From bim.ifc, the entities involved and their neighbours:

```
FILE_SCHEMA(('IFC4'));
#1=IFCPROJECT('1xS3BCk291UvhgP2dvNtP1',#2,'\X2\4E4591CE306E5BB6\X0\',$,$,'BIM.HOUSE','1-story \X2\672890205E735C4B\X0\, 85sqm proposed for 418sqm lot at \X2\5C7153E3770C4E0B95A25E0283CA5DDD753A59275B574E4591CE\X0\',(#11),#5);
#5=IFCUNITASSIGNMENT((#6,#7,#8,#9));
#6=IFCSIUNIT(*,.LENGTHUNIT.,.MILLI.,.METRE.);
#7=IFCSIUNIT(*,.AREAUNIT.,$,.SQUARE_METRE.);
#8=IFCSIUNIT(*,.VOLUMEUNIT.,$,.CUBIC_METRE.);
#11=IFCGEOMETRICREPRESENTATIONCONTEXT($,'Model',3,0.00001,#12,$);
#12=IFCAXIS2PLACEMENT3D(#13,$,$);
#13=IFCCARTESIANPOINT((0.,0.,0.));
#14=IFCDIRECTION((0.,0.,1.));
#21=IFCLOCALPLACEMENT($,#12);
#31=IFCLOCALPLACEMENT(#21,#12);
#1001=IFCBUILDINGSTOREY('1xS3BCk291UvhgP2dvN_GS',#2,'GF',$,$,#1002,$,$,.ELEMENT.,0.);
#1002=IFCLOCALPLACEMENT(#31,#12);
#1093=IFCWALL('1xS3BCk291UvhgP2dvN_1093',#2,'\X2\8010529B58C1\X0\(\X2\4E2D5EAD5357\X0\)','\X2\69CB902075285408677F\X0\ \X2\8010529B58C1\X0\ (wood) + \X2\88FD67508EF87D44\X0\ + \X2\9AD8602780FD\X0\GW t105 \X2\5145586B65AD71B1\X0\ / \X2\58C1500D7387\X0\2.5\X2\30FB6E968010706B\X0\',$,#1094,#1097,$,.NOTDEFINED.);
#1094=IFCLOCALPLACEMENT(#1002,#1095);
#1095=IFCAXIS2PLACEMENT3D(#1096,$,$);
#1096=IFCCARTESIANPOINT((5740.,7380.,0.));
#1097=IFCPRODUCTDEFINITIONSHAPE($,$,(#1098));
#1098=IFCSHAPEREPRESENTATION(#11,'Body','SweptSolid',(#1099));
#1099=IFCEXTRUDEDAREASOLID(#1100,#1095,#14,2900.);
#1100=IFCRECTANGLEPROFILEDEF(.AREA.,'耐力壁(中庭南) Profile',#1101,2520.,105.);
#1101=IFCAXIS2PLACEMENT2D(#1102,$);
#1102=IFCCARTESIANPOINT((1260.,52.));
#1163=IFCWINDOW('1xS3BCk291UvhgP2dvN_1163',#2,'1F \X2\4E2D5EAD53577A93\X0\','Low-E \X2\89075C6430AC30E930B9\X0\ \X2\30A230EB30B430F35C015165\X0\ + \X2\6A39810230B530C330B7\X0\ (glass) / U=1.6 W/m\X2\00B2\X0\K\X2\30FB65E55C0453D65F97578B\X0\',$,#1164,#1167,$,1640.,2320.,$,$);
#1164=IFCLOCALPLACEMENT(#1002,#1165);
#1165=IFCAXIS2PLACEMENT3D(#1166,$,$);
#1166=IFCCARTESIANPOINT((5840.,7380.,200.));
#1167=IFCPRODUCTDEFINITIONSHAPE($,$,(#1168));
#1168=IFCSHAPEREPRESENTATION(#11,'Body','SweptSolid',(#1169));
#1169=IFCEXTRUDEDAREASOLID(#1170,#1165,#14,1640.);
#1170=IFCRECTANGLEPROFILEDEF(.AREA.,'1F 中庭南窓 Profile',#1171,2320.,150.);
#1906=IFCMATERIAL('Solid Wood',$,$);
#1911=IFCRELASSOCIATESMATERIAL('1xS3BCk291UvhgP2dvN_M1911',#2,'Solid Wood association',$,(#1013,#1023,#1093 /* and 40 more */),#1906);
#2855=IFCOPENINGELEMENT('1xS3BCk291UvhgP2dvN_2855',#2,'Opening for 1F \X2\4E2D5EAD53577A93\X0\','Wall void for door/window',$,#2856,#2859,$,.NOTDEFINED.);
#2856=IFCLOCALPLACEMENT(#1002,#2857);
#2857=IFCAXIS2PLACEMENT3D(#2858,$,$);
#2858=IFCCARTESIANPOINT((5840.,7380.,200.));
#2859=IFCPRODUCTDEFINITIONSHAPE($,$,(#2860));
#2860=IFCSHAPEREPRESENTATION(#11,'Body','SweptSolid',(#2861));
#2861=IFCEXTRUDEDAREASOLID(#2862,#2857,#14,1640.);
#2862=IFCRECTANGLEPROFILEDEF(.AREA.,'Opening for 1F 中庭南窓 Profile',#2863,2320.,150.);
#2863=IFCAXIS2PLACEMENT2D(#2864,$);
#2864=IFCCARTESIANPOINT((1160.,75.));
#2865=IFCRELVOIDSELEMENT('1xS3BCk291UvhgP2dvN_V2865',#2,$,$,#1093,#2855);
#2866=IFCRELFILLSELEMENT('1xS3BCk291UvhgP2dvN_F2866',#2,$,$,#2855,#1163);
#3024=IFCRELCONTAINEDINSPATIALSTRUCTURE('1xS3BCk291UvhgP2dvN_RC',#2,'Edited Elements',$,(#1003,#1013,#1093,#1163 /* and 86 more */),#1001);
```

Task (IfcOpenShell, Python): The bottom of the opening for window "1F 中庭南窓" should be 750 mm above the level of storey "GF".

```python
import numpy as np
import ifcopenshell
import ifcopenshell.api.geometry
import ifcopenshell.geom
import ifcopenshell.util.element
import ifcopenshell.util.placement
import ifcopenshell.util.shape
import ifcopenshell.util.unit

model = ifcopenshell.open("bim.ifc")
unit_scale = ifcopenshell.util.unit.calculate_unit_scale(model)

window = model.by_id(1163)
opening = window.FillsVoids[0].RelatingOpeningElement
storey = ifcopenshell.util.element.get_container(window, ifc_class="IfcBuildingStorey")
level = ifcopenshell.util.placement.get_local_placement(storey.ObjectPlacement)[2, 3]

# The opening's origin need not be at the sill, so measure its lowest point.
shape = ifcopenshell.geom.create_shape(ifcopenshell.geom.settings(), opening)
bottom = ifcopenshell.util.shape.get_shape_bottom_elevation(shape, shape.geometry) / unit_scale
dz = level + 0.75 / unit_scale - bottom

shift = np.array([0.0, 0.0, dz])
# The window is not placed relative to its opening, so move both.
for product in (opening, window):
    matrix = ifcopenshell.util.placement.get_local_placement(product.ObjectPlacement)
    matrix[:3, 3] += shift
    ifcopenshell.api.geometry.edit_object_placement(model, product=product, matrix=matrix, is_si=False)

print(f"moved by {dz * unit_scale:+.3f} m")

model.write("bim_edited.ifc")
```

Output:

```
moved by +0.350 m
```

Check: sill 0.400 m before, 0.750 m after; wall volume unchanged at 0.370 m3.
